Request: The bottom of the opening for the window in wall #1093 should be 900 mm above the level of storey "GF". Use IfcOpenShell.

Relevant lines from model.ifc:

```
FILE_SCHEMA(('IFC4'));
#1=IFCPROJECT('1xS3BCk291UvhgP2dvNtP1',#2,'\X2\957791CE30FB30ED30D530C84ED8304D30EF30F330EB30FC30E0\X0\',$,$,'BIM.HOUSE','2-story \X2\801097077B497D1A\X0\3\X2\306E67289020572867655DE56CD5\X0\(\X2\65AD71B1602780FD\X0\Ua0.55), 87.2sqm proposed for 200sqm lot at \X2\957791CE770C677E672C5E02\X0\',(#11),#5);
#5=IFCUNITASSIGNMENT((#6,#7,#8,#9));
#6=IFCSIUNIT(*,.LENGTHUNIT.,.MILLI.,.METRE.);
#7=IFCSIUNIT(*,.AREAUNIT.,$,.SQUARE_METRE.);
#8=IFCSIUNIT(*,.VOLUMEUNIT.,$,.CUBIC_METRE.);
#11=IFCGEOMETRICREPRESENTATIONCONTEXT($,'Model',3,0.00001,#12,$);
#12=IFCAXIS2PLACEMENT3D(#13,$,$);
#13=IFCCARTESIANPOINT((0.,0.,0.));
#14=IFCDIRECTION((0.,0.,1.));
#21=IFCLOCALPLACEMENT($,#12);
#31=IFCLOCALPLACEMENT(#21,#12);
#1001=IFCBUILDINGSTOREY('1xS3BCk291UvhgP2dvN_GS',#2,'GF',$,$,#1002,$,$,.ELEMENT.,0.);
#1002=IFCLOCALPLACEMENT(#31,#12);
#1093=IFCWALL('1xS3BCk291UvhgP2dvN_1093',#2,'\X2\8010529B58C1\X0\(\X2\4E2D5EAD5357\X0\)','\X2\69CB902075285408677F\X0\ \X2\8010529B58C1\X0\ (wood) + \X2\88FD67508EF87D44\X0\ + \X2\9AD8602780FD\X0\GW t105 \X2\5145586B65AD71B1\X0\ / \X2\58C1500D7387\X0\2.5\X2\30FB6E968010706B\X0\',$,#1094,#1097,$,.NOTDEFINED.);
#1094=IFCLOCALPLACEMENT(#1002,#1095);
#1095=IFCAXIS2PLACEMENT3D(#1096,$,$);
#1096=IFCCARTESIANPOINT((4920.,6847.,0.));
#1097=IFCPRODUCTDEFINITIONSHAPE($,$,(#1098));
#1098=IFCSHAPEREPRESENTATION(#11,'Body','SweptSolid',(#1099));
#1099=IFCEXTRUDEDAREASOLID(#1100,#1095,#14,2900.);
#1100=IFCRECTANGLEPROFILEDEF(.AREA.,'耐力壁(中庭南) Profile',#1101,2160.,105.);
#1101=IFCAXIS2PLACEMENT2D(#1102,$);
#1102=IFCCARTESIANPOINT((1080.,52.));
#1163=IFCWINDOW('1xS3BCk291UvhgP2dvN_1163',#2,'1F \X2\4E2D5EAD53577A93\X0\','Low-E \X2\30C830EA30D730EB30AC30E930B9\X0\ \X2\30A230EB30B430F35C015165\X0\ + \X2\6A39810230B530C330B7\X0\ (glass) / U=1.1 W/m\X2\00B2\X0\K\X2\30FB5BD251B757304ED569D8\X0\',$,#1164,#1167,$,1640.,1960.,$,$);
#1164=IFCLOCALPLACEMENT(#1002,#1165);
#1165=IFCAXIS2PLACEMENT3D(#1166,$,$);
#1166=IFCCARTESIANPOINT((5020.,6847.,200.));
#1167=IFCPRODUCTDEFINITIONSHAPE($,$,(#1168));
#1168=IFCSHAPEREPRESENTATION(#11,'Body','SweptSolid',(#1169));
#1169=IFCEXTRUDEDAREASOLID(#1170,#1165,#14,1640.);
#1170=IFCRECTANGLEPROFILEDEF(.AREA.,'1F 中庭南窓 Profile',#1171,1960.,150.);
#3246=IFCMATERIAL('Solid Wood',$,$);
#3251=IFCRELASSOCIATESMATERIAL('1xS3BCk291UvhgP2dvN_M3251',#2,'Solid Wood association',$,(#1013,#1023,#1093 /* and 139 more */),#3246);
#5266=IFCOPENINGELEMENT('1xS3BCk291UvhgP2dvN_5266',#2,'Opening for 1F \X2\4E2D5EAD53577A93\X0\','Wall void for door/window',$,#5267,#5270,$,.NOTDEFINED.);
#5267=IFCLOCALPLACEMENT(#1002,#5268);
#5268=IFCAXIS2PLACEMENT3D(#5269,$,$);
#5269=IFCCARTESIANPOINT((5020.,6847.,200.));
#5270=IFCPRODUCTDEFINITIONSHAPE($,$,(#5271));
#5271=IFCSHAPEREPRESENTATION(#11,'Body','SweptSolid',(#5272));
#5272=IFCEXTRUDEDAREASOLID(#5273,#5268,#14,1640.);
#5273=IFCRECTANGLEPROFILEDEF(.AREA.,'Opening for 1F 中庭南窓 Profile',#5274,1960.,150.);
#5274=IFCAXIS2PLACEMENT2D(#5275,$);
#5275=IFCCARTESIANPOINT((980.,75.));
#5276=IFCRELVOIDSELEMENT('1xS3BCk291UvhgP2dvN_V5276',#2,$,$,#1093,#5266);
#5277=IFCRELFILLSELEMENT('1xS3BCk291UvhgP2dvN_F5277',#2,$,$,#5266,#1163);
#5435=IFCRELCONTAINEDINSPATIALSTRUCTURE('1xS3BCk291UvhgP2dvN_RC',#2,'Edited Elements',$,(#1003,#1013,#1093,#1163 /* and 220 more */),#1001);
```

```python
import numpy as np
import ifcopenshell
import ifcopenshell.api.geometry
import ifcopenshell.geom
import ifcopenshell.util.element
import ifcopenshell.util.placement
import ifcopenshell.util.shape
import ifcopenshell.util.unit

model = ifcopenshell.open("model.ifc")
unit_scale = ifcopenshell.util.unit.calculate_unit_scale(model)

window = model.by_guid("1xS3BCk291UvhgP2dvN_1163")
opening = window.FillsVoids[0].RelatingOpeningElement
storey = ifcopenshell.util.element.get_container(window, ifc_class="IfcBuildingStorey")
level = ifcopenshell.util.placement.get_local_placement(storey.ObjectPlacement)[2, 3]

# The opening's origin need not be at the sill, so measure its lowest point.
shape = ifcopenshell.geom.create_shape(ifcopenshell.geom.settings(), opening)
bottom = ifcopenshell.util.shape.get_shape_bottom_elevation(shape, shape.geometry) / unit_scale
dz = level + 0.9 / unit_scale - bottom

shift = np.array([0.0, 0.0, dz])
# The window is not placed relative to its opening, so move both.
for product in (opening, window):
    matrix = ifcopenshell.util.placement.get_local_placement(product.ObjectPlacement)
    matrix[:3, 3] += shift
    ifcopenshell.api.geometry.edit_object_placement(model, product=product, matrix=matrix, is_si=False)

print(f"moved by {dz * unit_scale:+.3f} m")

model.write("model_v2.ifc")
```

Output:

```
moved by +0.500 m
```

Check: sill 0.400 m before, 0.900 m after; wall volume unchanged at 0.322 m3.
